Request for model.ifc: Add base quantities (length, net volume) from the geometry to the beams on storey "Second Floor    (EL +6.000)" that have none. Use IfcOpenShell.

First a look at what the model holds.

```python
import ifcopenshell
import ifcopenshell.util.element
import ifcopenshell.util.unit

model = ifcopenshell.open("model.ifc")
print(model.schema)
for unit_type in ("LENGTHUNIT", "AREAUNIT", "VOLUMEUNIT"):
    print(unit_type, ifcopenshell.util.unit.calculate_unit_scale(model, unit_type))
storey = next(s for s in model.by_type("IfcBuildingStorey") if s.Name == "Second Floor    (EL +6.000)")
beams = [e for e in ifcopenshell.util.element.get_decomposition(storey) if e.is_a("IfcBeam")]
for e in sorted(beams, key=lambda e: e.id()):
    print(e.id(), e.is_a(), e.Name, list(ifcopenshell.util.element.get_psets(e, qtos_only=True)), sep=" | ")
```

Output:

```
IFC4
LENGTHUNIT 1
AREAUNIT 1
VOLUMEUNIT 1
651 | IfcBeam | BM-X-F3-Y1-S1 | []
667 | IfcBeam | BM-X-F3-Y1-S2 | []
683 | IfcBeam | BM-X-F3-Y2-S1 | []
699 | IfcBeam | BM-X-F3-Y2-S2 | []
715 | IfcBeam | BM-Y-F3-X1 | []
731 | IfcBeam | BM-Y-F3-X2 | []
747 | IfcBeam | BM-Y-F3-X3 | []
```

```python
import ifcopenshell
import ifcopenshell.api.pset
import ifcopenshell.geom
import ifcopenshell.util.element
import ifcopenshell.util.shape
import ifcopenshell.util.unit

model = ifcopenshell.open("model.ifc")
unit_scale = ifcopenshell.util.unit.calculate_unit_scale(model)
volume_scale = ifcopenshell.util.unit.calculate_unit_scale(model, "VOLUMEUNIT")
settings = ifcopenshell.geom.settings()

storey = next(s for s in model.by_type("IfcBuildingStorey") if s.Name == "Second Floor    (EL +6.000)")
beams = [e for e in ifcopenshell.util.element.get_decomposition(storey) if e.is_a("IfcBeam")]

for e in sorted(beams, key=lambda e: e.id()):
    if ifcopenshell.util.element.get_psets(e, qtos_only=True, should_inherit=False):
        continue
    # Geometry comes back in metres, in the element's own axes.
    shape = ifcopenshell.geom.create_shape(settings, e)
    values = {
        "Length": ifcopenshell.util.shape.get_max_xyz(shape.geometry) / unit_scale,
        "NetVolume": ifcopenshell.util.shape.get_volume(shape.geometry) / volume_scale,
    }
    qto = ifcopenshell.api.pset.add_qto(model, product=e, name="Qto_BeamBaseQuantities")
    ifcopenshell.api.pset.edit_qto(model, qto=qto, properties=values)
    print(e.id(), {k: round(v, 3) for k, v in values.items()})

model.write("model_updated.ifc")
```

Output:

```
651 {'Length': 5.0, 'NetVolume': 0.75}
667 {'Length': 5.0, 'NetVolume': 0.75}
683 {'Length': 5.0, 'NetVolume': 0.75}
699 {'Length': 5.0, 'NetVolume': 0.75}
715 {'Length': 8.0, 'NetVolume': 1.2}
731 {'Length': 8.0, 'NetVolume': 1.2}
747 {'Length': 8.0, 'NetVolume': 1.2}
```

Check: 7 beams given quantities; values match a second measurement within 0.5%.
